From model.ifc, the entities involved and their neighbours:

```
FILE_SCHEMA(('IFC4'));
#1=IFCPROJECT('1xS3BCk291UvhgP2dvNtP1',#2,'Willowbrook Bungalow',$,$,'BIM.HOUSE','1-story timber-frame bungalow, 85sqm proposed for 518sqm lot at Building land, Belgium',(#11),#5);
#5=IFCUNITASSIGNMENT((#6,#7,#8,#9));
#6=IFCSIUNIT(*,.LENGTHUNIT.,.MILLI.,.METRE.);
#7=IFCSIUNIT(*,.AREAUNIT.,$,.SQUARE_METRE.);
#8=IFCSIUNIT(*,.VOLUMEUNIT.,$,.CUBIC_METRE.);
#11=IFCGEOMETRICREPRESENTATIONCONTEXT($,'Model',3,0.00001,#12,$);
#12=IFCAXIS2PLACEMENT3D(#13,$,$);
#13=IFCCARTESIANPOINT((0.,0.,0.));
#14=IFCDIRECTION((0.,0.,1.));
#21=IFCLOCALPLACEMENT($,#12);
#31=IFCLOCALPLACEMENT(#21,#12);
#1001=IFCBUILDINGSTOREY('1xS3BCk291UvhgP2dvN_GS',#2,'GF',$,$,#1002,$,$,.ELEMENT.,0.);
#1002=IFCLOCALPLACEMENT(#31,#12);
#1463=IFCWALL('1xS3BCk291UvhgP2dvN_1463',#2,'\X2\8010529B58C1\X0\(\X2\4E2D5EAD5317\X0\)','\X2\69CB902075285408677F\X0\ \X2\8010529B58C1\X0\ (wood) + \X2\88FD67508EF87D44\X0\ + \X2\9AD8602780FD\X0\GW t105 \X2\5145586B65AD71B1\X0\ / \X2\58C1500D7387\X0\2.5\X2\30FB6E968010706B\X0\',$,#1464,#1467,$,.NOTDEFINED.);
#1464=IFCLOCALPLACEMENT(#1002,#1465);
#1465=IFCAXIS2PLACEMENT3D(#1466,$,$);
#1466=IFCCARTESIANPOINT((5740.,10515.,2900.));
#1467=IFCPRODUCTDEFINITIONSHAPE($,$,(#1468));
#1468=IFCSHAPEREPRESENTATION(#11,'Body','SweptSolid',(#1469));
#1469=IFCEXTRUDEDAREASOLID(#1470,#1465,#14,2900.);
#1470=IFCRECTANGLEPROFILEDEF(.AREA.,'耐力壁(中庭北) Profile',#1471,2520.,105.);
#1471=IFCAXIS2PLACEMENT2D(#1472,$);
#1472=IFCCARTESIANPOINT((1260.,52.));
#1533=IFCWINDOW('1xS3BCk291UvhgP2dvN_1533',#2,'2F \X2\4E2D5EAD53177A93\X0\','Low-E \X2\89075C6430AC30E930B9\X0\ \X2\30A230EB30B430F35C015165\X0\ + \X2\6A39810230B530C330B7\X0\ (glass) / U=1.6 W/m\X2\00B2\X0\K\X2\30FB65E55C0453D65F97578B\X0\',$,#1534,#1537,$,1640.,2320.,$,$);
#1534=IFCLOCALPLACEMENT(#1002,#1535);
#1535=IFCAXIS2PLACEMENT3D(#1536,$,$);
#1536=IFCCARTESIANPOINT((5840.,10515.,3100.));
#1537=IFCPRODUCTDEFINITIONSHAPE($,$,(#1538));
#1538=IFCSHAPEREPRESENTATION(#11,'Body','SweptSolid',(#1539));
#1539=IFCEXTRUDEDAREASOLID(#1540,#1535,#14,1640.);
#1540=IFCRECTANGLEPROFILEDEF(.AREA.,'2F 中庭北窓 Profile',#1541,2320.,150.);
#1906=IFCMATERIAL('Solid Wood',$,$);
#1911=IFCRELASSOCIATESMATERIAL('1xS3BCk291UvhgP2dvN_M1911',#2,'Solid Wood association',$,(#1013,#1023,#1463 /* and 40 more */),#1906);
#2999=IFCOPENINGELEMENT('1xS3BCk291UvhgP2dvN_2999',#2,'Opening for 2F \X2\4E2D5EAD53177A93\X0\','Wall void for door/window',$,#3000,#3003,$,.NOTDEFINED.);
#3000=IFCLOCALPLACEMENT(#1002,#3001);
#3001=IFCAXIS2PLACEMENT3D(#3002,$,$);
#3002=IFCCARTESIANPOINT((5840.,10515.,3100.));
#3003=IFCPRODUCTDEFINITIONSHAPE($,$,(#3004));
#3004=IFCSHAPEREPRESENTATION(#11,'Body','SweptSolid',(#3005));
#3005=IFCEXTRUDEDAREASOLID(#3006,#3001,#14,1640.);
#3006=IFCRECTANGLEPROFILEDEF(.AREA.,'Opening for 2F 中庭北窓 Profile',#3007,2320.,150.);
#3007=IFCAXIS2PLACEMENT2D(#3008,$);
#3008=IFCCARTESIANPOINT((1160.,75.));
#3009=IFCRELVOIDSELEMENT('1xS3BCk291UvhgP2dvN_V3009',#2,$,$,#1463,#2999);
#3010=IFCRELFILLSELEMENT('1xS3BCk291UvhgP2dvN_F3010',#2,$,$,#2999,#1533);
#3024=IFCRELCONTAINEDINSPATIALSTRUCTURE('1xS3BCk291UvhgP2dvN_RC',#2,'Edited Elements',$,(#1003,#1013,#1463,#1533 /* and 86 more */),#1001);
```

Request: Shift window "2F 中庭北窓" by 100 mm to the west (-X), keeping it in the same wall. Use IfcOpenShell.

```python
import ifcopenshell
import ifcopenshell.api.geometry
import ifcopenshell.util.placement
import ifcopenshell.util.unit

model = ifcopenshell.open("model.ifc")
unit_scale = ifcopenshell.util.unit.calculate_unit_scale(model)

window = model.by_id(1533)
opening = window.FillsVoids[0].RelatingOpeningElement
wall = opening.VoidsElements[0].RelatingBuildingElement

wall_matrix = ifcopenshell.util.placement.get_local_placement(wall.ObjectPlacement)
shift = wall_matrix[:3, 0] * -0.1 / unit_scale
before = ifcopenshell.util.placement.get_local_placement(window.ObjectPlacement)[:3, 3].copy()

# The window is not placed relative to its opening, so move both.
for product in (opening, window):
    matrix = ifcopenshell.util.placement.get_local_placement(product.ObjectPlacement)
    matrix[:3, 3] += shift
    ifcopenshell.api.geometry.edit_object_placement(model, product=product, matrix=matrix, is_si=False)

after = ifcopenshell.util.placement.get_local_placement(window.ObjectPlacement)[:3, 3]
print("window moved by", (after - before).round(3) + 0.0)

model.write("model_v2.ifc")
```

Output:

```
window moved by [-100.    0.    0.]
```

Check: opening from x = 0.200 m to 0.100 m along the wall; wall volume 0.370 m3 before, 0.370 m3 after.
